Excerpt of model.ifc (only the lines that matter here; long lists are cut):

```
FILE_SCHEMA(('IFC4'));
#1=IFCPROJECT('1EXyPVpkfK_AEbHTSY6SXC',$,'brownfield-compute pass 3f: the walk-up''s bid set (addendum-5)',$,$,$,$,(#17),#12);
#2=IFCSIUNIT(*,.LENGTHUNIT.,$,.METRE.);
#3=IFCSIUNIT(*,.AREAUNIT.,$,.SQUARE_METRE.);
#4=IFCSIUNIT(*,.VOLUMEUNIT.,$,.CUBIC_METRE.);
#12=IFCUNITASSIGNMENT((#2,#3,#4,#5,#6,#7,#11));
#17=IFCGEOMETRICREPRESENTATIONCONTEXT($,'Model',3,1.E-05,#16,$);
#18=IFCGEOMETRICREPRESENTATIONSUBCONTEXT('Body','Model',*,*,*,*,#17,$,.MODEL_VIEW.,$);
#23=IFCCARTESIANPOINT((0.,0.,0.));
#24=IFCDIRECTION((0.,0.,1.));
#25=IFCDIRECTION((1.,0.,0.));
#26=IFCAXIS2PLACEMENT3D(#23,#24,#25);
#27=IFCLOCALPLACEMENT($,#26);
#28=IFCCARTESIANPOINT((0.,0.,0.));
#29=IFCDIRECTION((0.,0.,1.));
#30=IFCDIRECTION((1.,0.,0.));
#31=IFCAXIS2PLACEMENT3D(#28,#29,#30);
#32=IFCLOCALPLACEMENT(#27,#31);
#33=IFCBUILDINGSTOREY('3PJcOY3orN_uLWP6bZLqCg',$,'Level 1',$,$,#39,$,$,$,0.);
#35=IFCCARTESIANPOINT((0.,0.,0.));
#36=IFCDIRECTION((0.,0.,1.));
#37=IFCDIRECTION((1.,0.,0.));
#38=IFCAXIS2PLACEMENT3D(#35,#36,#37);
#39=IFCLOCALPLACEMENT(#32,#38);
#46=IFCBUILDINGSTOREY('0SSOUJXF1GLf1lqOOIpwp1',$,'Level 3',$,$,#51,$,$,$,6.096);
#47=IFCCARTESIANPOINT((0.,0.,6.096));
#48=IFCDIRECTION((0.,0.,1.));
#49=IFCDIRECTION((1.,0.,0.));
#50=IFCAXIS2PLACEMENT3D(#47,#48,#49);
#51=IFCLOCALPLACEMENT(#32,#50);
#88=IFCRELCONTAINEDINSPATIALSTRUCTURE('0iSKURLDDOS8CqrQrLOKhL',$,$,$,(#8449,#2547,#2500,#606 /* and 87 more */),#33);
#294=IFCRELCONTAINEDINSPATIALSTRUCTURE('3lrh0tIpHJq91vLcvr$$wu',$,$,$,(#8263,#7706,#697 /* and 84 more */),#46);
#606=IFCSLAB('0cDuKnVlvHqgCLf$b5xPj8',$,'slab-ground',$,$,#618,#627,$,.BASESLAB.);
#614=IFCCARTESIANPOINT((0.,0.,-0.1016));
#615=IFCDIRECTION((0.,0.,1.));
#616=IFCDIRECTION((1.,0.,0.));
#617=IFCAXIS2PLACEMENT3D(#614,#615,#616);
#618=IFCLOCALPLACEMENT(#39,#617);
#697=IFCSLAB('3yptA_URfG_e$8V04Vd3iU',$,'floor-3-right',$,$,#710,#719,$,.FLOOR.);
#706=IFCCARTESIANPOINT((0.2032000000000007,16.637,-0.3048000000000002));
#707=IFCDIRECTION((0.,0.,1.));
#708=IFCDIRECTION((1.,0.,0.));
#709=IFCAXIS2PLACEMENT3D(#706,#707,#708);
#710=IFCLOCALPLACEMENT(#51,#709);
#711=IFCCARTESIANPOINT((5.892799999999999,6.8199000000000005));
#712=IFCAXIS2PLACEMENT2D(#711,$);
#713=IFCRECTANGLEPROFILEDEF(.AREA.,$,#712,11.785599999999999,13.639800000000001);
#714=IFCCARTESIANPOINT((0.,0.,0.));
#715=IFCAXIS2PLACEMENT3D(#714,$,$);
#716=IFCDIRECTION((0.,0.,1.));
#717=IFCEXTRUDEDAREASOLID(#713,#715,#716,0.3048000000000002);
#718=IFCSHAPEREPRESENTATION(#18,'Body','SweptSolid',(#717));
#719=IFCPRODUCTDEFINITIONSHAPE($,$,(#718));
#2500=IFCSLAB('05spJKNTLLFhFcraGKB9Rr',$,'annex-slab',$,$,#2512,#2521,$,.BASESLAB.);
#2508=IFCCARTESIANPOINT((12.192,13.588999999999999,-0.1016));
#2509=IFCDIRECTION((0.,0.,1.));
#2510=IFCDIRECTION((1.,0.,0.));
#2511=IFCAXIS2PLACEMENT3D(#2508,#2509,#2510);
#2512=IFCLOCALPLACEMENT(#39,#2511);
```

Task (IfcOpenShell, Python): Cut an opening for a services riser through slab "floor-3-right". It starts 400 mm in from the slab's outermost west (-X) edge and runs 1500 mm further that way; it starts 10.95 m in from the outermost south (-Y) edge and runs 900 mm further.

```python
import numpy as np
import ifcopenshell
import ifcopenshell.api.feature
import ifcopenshell.api.geometry
import ifcopenshell.api.root
import ifcopenshell.geom
import ifcopenshell.util.placement
import ifcopenshell.util.representation
import ifcopenshell.util.shape
import ifcopenshell.util.unit

model = ifcopenshell.open("model.ifc")
unit_scale = ifcopenshell.util.unit.calculate_unit_scale(model)
settings = ifcopenshell.geom.settings()


def volume(element):
    """Net volume in cubic metres, openings subtracted."""
    shape = ifcopenshell.geom.create_shape(settings, element)
    return ifcopenshell.util.shape.get_volume(shape.geometry)


slab = model.by_guid("3yptA_URfG_e$8V04Vd3iU")
before = volume(slab)

# Extent in the slab's own axes, in metres. The edges named are its -X and -Y sides.
slab_shape = ifcopenshell.geom.create_shape(settings, slab)
vertices = ifcopenshell.util.shape.get_vertices(slab_shape.geometry)
x_min, y_min, bottom = vertices.min(axis=0)
top = vertices[:, 2].max()

opening = ifcopenshell.api.root.create_entity(model, ifc_class="IfcOpeningElement", name="Services riser opening", predefined_type="OPENING")
context = ifcopenshell.util.representation.get_context(model, "Model", "Body", "MODEL_VIEW")
width, depth = 1.5, 0.9
outline = [(0.0, 0.0), (width, 0.0), (width, depth), (0.0, depth), (0.0, 0.0)]
# Overshoot both faces by 50 mm so the cut is clean.
shape = ifcopenshell.api.geometry.add_slab_representation(
    model, context=context, depth=top - bottom + 0.1, polyline=outline
)
ifcopenshell.api.geometry.assign_representation(model, product=opening, representation=shape)

matrix = ifcopenshell.util.placement.get_local_placement(slab.ObjectPlacement)
matrix[:, 3] = matrix @ np.append(np.array([x_min + 0.4, y_min + 10.95, bottom - 0.05]) / unit_scale, 1.0)
ifcopenshell.api.geometry.edit_object_placement(model, product=opening, matrix=matrix, is_si=False)
ifcopenshell.api.feature.add_feature(model, feature=opening, element=slab)

after = volume(slab)

print(f"slab volume {before:.3f} -> {after:.3f} m3")

model.write("model_updated.ifc")
```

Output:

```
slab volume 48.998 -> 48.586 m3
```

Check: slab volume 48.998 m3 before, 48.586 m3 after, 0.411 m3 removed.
